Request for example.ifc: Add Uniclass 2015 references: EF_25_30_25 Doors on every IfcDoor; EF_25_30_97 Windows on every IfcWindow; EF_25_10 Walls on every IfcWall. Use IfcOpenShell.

First a look at what the model holds.

```python
import ifcopenshell

model = ifcopenshell.open("example.ifc")
print(model.schema)
print("classifications:", [c.Name for c in model.by_type("IfcClassification")])
for ifc_class in ("IfcDoor", "IfcRoof", "IfcStair", "IfcWall", "IfcWindow"):
    print(ifc_class, len(model.by_type(ifc_class)))
```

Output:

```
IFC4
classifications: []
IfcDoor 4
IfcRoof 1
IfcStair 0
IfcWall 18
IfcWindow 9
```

```python
import ifcopenshell
import ifcopenshell.api.classification

model = ifcopenshell.open("example.ifc")

system = ifcopenshell.api.classification.add_classification(model, classification="Uniclass 2015")

codes = {
    "IfcDoor": ("EF_25_30_25", "Doors"),
    "IfcWindow": ("EF_25_30_97", "Windows"),
    "IfcWall": ("EF_25_10", "Walls"),
}
for ifc_class, (code, name) in codes.items():
    products = model.by_type(ifc_class)
    ifcopenshell.api.classification.add_reference(
        model, products=products, classification=system, identification=code, name=name
    )
    print(code, len(products))

model.write("example_edited.ifc")
```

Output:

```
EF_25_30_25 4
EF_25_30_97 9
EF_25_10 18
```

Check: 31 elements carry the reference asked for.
